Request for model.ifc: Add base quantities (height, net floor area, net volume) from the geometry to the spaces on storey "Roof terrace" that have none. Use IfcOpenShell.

First a look at what the model holds.

```python
import ifcopenshell
import ifcopenshell.util.element
import ifcopenshell.util.unit

model = ifcopenshell.open("model.ifc")
print(model.schema)
for unit_type in ("LENGTHUNIT", "AREAUNIT", "VOLUMEUNIT"):
    print(unit_type, ifcopenshell.util.unit.calculate_unit_scale(model, unit_type))
storey = next(s for s in model.by_type("IfcBuildingStorey") if s.Name == "Roof terrace")
spaces = [e for e in ifcopenshell.util.element.get_decomposition(storey) if e.is_a("IfcSpace")]
for e in sorted(spaces, key=lambda e: e.id()):
    print(e.id(), e.is_a(), e.Name, list(ifcopenshell.util.element.get_psets(e, qtos_only=True)), sep=" | ")
```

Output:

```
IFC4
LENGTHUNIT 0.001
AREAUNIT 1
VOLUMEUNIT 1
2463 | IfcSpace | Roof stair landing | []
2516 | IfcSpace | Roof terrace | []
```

```python
import ifcopenshell
import ifcopenshell.api.pset
import ifcopenshell.geom
import ifcopenshell.util.element
import ifcopenshell.util.shape
import ifcopenshell.util.unit

model = ifcopenshell.open("model.ifc")
unit_scale = ifcopenshell.util.unit.calculate_unit_scale(model)
area_scale = ifcopenshell.util.unit.calculate_unit_scale(model, "AREAUNIT")
volume_scale = ifcopenshell.util.unit.calculate_unit_scale(model, "VOLUMEUNIT")
settings = ifcopenshell.geom.settings()

storey = next(s for s in model.by_type("IfcBuildingStorey") if s.Name == "Roof terrace")
spaces = [e for e in ifcopenshell.util.element.get_decomposition(storey) if e.is_a("IfcSpace")]

for e in sorted(spaces, key=lambda e: e.id()):
    if ifcopenshell.util.element.get_psets(e, qtos_only=True, should_inherit=False):
        continue
    # Geometry comes back in metres, in the element's own axes.
    shape = ifcopenshell.geom.create_shape(settings, e)
    values = {
        "Height": ifcopenshell.util.shape.get_z(shape.geometry) / unit_scale,
        "NetFloorArea": ifcopenshell.util.shape.get_footprint_area(shape.geometry) / area_scale,
        "NetVolume": ifcopenshell.util.shape.get_volume(shape.geometry) / volume_scale,
    }
    qto = ifcopenshell.api.pset.add_qto(model, product=e, name="Qto_SpaceBaseQuantities")
    ifcopenshell.api.pset.edit_qto(model, qto=qto, properties=values)
    print(e.id(), {k: round(v, 3) for k, v in values.items()})

model.write("model_edited.ifc")
```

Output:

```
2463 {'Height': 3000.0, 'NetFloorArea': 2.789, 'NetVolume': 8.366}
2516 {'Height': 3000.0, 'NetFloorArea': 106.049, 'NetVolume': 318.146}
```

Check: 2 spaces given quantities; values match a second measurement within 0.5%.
